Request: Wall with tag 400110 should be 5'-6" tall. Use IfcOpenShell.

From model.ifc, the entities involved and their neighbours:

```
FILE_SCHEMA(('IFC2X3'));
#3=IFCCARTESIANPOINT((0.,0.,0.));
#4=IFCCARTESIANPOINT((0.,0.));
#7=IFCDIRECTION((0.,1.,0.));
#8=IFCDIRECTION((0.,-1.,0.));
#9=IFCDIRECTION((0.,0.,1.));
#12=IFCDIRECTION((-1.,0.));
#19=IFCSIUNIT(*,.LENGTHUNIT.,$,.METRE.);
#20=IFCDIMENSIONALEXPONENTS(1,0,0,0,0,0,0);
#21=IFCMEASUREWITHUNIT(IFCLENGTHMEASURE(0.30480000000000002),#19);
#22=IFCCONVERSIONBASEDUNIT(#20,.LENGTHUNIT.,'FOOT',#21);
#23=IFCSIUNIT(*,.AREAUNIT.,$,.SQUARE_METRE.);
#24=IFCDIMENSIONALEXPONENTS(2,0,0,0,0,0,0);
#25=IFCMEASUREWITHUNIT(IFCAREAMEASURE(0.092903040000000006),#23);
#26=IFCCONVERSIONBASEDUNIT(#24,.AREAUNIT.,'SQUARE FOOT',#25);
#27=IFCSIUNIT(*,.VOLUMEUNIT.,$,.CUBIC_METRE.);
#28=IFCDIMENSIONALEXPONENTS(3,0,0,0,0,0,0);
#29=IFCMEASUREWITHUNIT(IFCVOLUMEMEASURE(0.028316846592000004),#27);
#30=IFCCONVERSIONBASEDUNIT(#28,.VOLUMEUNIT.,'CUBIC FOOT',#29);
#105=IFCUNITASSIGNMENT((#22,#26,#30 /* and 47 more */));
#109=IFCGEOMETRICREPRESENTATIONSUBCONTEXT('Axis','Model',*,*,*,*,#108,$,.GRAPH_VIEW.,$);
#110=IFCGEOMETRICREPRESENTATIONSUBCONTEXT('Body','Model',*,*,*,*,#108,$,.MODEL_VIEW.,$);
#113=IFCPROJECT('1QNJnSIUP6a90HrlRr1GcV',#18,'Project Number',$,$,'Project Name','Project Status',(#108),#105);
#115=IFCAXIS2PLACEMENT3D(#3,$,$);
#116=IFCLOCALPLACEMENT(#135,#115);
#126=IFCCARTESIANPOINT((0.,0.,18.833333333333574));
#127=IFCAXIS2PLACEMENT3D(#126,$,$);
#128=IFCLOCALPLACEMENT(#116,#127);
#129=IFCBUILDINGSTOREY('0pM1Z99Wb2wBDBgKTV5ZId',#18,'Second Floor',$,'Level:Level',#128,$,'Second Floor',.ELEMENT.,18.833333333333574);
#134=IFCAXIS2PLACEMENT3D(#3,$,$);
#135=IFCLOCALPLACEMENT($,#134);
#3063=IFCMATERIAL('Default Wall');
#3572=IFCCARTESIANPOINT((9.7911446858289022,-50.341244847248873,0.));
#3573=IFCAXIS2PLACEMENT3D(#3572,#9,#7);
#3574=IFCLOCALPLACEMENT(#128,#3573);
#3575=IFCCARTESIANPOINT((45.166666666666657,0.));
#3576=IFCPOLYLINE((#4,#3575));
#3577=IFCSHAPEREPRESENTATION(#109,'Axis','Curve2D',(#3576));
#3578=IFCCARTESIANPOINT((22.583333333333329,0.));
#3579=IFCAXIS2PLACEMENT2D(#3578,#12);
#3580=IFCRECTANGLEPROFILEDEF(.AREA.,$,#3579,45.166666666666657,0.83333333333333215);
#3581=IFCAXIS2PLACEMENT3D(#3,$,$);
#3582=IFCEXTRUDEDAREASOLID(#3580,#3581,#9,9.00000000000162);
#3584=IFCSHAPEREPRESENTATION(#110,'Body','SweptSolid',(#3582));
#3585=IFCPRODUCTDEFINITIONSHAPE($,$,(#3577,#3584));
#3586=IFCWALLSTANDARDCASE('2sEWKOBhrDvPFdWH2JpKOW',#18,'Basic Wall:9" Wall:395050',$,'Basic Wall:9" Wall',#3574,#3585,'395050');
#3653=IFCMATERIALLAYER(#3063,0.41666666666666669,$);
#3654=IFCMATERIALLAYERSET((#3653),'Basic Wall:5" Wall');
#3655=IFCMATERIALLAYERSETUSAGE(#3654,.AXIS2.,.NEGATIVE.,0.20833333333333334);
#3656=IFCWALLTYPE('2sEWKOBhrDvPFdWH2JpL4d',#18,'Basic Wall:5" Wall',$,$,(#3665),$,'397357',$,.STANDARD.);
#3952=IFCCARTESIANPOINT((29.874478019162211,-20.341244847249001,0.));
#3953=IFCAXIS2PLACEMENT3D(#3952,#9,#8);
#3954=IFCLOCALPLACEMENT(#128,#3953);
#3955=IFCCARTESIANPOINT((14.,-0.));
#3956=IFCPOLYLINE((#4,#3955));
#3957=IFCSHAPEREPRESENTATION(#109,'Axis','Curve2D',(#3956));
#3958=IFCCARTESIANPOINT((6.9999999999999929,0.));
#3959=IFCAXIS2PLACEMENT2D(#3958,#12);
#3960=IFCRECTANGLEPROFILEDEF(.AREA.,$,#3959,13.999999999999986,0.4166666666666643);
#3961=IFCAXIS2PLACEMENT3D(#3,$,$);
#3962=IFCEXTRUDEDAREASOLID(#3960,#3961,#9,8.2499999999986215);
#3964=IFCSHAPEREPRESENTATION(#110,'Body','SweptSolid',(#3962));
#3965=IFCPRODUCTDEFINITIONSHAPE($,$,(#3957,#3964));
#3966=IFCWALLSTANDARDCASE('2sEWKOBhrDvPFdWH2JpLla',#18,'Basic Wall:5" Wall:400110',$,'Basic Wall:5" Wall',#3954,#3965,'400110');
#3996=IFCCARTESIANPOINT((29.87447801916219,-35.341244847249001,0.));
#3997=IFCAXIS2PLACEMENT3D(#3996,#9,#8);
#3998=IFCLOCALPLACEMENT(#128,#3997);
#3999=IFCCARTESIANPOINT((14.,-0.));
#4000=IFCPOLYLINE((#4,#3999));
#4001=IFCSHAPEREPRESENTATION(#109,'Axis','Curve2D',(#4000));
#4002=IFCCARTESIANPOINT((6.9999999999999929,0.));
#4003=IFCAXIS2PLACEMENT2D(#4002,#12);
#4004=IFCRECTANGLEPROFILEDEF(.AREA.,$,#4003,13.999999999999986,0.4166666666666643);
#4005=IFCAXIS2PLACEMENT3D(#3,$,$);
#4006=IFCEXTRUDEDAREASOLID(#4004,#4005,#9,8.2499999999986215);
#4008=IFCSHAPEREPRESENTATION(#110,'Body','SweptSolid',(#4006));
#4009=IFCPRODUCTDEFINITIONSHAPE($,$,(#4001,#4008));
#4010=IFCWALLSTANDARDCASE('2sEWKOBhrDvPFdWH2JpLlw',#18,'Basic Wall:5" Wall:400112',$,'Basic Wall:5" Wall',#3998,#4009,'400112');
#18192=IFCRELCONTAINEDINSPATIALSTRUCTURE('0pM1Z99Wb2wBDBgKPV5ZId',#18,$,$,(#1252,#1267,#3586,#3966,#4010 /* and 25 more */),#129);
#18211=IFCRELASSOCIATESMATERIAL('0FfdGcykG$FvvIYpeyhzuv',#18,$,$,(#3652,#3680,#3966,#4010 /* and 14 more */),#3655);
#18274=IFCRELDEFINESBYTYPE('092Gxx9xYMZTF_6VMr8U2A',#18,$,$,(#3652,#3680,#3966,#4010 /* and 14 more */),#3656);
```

```python
import ifcopenshell
import ifcopenshell.geom
import ifcopenshell.util.representation
import ifcopenshell.util.shape
import ifcopenshell.util.unit

model = ifcopenshell.open("model.ifc")
unit_scale = ifcopenshell.util.unit.calculate_unit_scale(model)
settings = ifcopenshell.geom.settings()


def volume(element):
    """Net volume in cubic metres, openings subtracted."""
    shape = ifcopenshell.geom.create_shape(settings, element)
    return ifcopenshell.util.shape.get_volume(shape.geometry)


wall = model.by_guid("2sEWKOBhrDvPFdWH2JpLla")
before = volume(wall)

body = ifcopenshell.util.representation.get_representation(wall, "Model", "Body")
solid = body.Items[0]
old_height = solid.Depth
solid.Depth = 66 * 0.0254 / unit_scale
after = volume(wall)

print(f"height {old_height:g} -> {solid.Depth:g}, volume {before:.3f} -> {after:.3f} m3")

model.write("model_edited.ifc")
```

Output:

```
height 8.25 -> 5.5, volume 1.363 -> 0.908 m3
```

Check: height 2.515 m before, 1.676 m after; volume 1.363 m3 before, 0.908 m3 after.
